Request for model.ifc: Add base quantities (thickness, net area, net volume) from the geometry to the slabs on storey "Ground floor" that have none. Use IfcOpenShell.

First a look at what the model holds.

```python
import ifcopenshell
import ifcopenshell.util.element
import ifcopenshell.util.unit

model = ifcopenshell.open("model.ifc")
print(model.schema)
for unit_type in ("LENGTHUNIT", "AREAUNIT", "VOLUMEUNIT"):
    print(unit_type, ifcopenshell.util.unit.calculate_unit_scale(model, unit_type))
storey = next(s for s in model.by_type("IfcBuildingStorey") if s.Name == "Ground floor")
slabs = [e for e in ifcopenshell.util.element.get_decomposition(storey) if e.is_a("IfcSlab")]
for e in sorted(slabs, key=lambda e: e.id()):
    print(e.id(), e.is_a(), e.Name, list(ifcopenshell.util.element.get_psets(e, qtos_only=True)), sep=" | ")
```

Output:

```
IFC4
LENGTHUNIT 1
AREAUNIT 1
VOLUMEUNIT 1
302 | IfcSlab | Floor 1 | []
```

```python
import ifcopenshell
import ifcopenshell.api.pset
import ifcopenshell.geom
import ifcopenshell.util.element
import ifcopenshell.util.shape
import ifcopenshell.util.unit

model = ifcopenshell.open("model.ifc")
unit_scale = ifcopenshell.util.unit.calculate_unit_scale(model)
area_scale = ifcopenshell.util.unit.calculate_unit_scale(model, "AREAUNIT")
volume_scale = ifcopenshell.util.unit.calculate_unit_scale(model, "VOLUMEUNIT")
settings = ifcopenshell.geom.settings()

storey = next(s for s in model.by_type("IfcBuildingStorey") if s.Name == "Ground floor")
slabs = [e for e in ifcopenshell.util.element.get_decomposition(storey) if e.is_a("IfcSlab")]

for e in sorted(slabs, key=lambda e: e.id()):
    if ifcopenshell.util.element.get_psets(e, qtos_only=True, should_inherit=False):
        continue
    # Geometry comes back in metres, in the element's own axes.
    shape = ifcopenshell.geom.create_shape(settings, e)
    values = {
        "Width": ifcopenshell.util.shape.get_z(shape.geometry) / unit_scale,
        "NetArea": ifcopenshell.util.shape.get_footprint_area(shape.geometry) / area_scale,
        "NetVolume": ifcopenshell.util.shape.get_volume(shape.geometry) / volume_scale,
    }
    qto = ifcopenshell.api.pset.add_qto(model, product=e, name="Qto_SlabBaseQuantities")
    ifcopenshell.api.pset.edit_qto(model, qto=qto, properties=values)
    print(e.id(), {k: round(v, 3) for k, v in values.items()})

model.write("model_v2.ifc")
```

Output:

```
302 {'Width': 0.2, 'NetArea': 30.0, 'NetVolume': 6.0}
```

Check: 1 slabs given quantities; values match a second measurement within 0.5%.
